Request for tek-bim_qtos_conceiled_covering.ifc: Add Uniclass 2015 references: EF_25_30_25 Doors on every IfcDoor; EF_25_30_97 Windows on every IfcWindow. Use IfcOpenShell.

First a look at what the model holds.

```python
import ifcopenshell

model = ifcopenshell.open("tek-bim_qtos_conceiled_covering.ifc")
print(model.schema)
print("classifications:", [c.Name for c in model.by_type("IfcClassification")])
for ifc_class in ("IfcDoor", "IfcRoof", "IfcStair", "IfcWall", "IfcWindow"):
    print(ifc_class, len(model.by_type(ifc_class)))
```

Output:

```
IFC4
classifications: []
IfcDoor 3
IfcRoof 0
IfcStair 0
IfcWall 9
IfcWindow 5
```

```python
import ifcopenshell
import ifcopenshell.api.classification

model = ifcopenshell.open("tek-bim_qtos_conceiled_covering.ifc")

system = ifcopenshell.api.classification.add_classification(model, classification="Uniclass 2015")

codes = {
    "IfcDoor": ("EF_25_30_25", "Doors"),
    "IfcWindow": ("EF_25_30_97", "Windows"),
}
for ifc_class, (code, name) in codes.items():
    products = model.by_type(ifc_class)
    ifcopenshell.api.classification.add_reference(
        model, products=products, classification=system, identification=code, name=name
    )
    print(code, len(products))

model.write("tek-bim_qtos_conceiled_covering_v2.ifc")
```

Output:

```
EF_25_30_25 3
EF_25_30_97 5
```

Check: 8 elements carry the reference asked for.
